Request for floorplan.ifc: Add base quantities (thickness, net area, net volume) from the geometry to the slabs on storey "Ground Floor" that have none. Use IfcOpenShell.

First a look at what the model holds.

```python
import ifcopenshell
import ifcopenshell.util.element
import ifcopenshell.util.unit

model = ifcopenshell.open("floorplan.ifc")
print(model.schema)
for unit_type in ("LENGTHUNIT", "AREAUNIT", "VOLUMEUNIT"):
    print(unit_type, ifcopenshell.util.unit.calculate_unit_scale(model, unit_type))
storey = next(s for s in model.by_type("IfcBuildingStorey") if s.Name == "Ground Floor")
slabs = [e for e in ifcopenshell.util.element.get_decomposition(storey) if e.is_a("IfcSlab")]
for e in sorted(slabs, key=lambda e: e.id()):
    print(e.id(), e.is_a(), e.Name, list(ifcopenshell.util.element.get_psets(e, qtos_only=True)), sep=" | ")
```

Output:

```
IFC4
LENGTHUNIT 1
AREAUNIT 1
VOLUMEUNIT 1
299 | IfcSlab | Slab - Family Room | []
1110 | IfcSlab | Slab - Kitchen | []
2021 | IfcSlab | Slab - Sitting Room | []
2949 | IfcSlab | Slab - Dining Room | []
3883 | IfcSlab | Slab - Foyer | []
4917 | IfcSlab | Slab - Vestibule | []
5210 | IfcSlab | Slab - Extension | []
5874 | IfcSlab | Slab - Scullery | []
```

```python
import ifcopenshell
import ifcopenshell.api.pset
import ifcopenshell.geom
import ifcopenshell.util.element
import ifcopenshell.util.shape
import ifcopenshell.util.unit

model = ifcopenshell.open("floorplan.ifc")
unit_scale = ifcopenshell.util.unit.calculate_unit_scale(model)
area_scale = ifcopenshell.util.unit.calculate_unit_scale(model, "AREAUNIT")
volume_scale = ifcopenshell.util.unit.calculate_unit_scale(model, "VOLUMEUNIT")
settings = ifcopenshell.geom.settings()

storey = next(s for s in model.by_type("IfcBuildingStorey") if s.Name == "Ground Floor")
slabs = [e for e in ifcopenshell.util.element.get_decomposition(storey) if e.is_a("IfcSlab")]

for e in sorted(slabs, key=lambda e: e.id()):
    if ifcopenshell.util.element.get_psets(e, qtos_only=True, should_inherit=False):
        continue
    # Geometry comes back in metres, in the element's own axes.
    shape = ifcopenshell.geom.create_shape(settings, e)
    values = {
        "Width": ifcopenshell.util.shape.get_z(shape.geometry) / unit_scale,
        "NetArea": ifcopenshell.util.shape.get_footprint_area(shape.geometry) / area_scale,
        "NetVolume": ifcopenshell.util.shape.get_volume(shape.geometry) / volume_scale,
    }
    qto = ifcopenshell.api.pset.add_qto(model, product=e, name="Qto_SlabBaseQuantities")
    ifcopenshell.api.pset.edit_qto(model, qto=qto, properties=values)
    print(e.id(), {k: round(v, 3) for k, v in values.items()})

model.write("floorplan_updated.ifc")
```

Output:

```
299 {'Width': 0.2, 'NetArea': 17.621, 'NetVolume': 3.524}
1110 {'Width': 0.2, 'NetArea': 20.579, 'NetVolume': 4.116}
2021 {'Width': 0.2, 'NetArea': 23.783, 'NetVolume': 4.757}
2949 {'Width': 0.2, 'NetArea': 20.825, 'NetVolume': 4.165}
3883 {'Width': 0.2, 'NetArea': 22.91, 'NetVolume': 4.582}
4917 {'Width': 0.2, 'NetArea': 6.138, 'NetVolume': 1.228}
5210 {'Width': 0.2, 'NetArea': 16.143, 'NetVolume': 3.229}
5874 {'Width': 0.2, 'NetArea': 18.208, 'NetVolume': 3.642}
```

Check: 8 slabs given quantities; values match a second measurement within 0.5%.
